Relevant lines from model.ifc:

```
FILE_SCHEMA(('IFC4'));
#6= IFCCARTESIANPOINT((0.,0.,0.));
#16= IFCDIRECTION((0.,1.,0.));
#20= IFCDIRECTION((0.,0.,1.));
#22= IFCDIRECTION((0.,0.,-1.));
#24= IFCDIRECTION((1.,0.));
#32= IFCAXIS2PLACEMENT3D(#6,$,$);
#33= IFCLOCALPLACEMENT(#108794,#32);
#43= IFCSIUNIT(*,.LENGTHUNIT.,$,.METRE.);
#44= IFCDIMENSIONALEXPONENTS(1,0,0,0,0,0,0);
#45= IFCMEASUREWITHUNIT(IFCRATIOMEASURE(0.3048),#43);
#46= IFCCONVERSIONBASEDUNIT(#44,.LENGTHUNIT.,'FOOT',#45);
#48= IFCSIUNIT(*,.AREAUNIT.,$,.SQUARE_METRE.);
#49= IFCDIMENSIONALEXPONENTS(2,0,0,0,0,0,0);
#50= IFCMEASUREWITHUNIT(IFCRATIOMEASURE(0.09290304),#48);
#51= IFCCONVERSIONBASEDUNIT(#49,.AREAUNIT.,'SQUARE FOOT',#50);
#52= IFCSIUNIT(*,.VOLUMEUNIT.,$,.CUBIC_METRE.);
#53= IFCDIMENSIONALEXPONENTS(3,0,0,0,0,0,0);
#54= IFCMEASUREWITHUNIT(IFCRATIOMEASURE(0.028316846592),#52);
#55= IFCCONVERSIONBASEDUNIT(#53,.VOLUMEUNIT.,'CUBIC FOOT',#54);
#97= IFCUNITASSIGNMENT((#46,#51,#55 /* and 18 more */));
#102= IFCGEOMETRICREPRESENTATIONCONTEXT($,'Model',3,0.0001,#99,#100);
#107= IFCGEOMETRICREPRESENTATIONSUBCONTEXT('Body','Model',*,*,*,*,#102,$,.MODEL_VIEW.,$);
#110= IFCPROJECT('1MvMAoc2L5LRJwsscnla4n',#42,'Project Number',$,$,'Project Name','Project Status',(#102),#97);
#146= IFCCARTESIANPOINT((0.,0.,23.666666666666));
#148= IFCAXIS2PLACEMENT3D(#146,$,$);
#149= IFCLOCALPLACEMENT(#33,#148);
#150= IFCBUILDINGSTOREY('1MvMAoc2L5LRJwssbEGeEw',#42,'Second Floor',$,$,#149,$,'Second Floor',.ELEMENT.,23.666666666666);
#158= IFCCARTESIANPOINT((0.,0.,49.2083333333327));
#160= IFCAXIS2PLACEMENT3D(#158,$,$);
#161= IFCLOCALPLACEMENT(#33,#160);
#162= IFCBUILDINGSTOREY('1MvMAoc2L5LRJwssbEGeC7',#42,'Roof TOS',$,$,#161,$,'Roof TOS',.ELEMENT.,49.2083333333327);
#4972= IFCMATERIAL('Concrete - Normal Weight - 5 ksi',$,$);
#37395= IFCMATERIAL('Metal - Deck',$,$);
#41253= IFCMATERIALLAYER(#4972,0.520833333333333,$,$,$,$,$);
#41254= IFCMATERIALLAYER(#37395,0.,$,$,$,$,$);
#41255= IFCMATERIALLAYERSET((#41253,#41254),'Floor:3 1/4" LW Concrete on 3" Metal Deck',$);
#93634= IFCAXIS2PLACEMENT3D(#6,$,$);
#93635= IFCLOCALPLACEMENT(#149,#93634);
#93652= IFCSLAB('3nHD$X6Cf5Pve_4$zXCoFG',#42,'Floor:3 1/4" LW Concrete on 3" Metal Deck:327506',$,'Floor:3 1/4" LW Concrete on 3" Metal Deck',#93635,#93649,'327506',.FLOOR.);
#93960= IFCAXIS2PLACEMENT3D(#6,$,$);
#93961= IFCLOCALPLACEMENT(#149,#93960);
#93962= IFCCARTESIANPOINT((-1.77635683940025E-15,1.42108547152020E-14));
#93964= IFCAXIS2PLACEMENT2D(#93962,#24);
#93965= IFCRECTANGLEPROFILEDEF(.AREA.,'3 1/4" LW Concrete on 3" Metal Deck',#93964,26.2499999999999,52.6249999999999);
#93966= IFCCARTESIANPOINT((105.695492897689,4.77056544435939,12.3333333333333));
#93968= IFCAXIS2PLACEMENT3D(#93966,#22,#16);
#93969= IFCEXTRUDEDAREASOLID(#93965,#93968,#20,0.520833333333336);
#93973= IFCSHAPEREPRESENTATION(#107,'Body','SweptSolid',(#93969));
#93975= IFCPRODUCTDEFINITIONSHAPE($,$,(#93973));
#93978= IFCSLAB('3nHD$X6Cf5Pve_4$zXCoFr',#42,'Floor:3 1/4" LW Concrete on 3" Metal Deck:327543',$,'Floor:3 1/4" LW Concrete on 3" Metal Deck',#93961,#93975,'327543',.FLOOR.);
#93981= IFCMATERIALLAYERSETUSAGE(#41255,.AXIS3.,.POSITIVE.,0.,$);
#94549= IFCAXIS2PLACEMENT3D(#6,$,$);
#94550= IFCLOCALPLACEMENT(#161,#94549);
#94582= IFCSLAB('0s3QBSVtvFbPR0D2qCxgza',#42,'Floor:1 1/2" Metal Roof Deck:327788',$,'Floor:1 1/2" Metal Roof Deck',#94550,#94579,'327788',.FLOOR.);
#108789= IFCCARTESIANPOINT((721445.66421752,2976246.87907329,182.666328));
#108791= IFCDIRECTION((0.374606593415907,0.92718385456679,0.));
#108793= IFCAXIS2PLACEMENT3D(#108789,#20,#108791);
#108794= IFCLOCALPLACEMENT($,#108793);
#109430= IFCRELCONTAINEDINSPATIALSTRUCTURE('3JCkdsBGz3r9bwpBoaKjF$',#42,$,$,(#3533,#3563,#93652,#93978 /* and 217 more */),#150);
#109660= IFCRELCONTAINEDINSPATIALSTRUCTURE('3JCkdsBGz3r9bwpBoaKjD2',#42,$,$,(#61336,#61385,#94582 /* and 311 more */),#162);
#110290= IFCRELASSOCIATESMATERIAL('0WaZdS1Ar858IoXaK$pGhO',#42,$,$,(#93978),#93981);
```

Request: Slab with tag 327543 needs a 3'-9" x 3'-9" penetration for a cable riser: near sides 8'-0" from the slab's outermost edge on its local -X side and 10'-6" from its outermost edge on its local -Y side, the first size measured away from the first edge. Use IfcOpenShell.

```python
import numpy as np
import ifcopenshell
import ifcopenshell.api.feature
import ifcopenshell.api.geometry
import ifcopenshell.api.root
import ifcopenshell.geom
import ifcopenshell.util.placement
import ifcopenshell.util.representation
import ifcopenshell.util.shape
import ifcopenshell.util.unit

model = ifcopenshell.open("model.ifc")
unit_scale = ifcopenshell.util.unit.calculate_unit_scale(model)
settings = ifcopenshell.geom.settings()


def volume(element):
    """Net volume in cubic metres, openings subtracted."""
    shape = ifcopenshell.geom.create_shape(settings, element)
    return ifcopenshell.util.shape.get_volume(shape.geometry)


slab = model.by_guid("3nHD$X6Cf5Pve_4$zXCoFr")
before = volume(slab)

# Extent in the slab's own axes, in metres. The edges named are its -X and -Y sides.
slab_shape = ifcopenshell.geom.create_shape(settings, slab)
vertices = ifcopenshell.util.shape.get_vertices(slab_shape.geometry)
x_min, y_min, bottom = vertices.min(axis=0)
top = vertices[:, 2].max()

opening = ifcopenshell.api.root.create_entity(model, ifc_class="IfcOpeningElement", name="Cable riser opening", predefined_type="OPENING")
context = ifcopenshell.util.representation.get_context(model, "Model", "Body", "MODEL_VIEW")
width, depth = 1.143, 1.143
outline = [(0.0, 0.0), (width, 0.0), (width, depth), (0.0, depth), (0.0, 0.0)]
# Overshoot both faces by 50 mm so the cut is clean.
shape = ifcopenshell.api.geometry.add_slab_representation(
    model, context=context, depth=top - bottom + 0.1, polyline=outline
)
ifcopenshell.api.geometry.assign_representation(model, product=opening, representation=shape)

matrix = ifcopenshell.util.placement.get_local_placement(slab.ObjectPlacement)
matrix[:, 3] = matrix @ np.append(np.array([x_min + 2.4384, y_min + 3.2004, bottom - 0.05]) / unit_scale, 1.0)
ifcopenshell.api.geometry.edit_object_placement(model, product=opening, matrix=matrix, is_si=False)
ifcopenshell.api.feature.add_feature(model, feature=opening, element=slab)

after = volume(slab)

print(f"slab volume {before:.3f} -> {after:.3f} m3")

model.write("model_edited.ifc")
```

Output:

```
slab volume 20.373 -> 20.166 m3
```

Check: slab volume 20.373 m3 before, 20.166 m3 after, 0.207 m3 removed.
